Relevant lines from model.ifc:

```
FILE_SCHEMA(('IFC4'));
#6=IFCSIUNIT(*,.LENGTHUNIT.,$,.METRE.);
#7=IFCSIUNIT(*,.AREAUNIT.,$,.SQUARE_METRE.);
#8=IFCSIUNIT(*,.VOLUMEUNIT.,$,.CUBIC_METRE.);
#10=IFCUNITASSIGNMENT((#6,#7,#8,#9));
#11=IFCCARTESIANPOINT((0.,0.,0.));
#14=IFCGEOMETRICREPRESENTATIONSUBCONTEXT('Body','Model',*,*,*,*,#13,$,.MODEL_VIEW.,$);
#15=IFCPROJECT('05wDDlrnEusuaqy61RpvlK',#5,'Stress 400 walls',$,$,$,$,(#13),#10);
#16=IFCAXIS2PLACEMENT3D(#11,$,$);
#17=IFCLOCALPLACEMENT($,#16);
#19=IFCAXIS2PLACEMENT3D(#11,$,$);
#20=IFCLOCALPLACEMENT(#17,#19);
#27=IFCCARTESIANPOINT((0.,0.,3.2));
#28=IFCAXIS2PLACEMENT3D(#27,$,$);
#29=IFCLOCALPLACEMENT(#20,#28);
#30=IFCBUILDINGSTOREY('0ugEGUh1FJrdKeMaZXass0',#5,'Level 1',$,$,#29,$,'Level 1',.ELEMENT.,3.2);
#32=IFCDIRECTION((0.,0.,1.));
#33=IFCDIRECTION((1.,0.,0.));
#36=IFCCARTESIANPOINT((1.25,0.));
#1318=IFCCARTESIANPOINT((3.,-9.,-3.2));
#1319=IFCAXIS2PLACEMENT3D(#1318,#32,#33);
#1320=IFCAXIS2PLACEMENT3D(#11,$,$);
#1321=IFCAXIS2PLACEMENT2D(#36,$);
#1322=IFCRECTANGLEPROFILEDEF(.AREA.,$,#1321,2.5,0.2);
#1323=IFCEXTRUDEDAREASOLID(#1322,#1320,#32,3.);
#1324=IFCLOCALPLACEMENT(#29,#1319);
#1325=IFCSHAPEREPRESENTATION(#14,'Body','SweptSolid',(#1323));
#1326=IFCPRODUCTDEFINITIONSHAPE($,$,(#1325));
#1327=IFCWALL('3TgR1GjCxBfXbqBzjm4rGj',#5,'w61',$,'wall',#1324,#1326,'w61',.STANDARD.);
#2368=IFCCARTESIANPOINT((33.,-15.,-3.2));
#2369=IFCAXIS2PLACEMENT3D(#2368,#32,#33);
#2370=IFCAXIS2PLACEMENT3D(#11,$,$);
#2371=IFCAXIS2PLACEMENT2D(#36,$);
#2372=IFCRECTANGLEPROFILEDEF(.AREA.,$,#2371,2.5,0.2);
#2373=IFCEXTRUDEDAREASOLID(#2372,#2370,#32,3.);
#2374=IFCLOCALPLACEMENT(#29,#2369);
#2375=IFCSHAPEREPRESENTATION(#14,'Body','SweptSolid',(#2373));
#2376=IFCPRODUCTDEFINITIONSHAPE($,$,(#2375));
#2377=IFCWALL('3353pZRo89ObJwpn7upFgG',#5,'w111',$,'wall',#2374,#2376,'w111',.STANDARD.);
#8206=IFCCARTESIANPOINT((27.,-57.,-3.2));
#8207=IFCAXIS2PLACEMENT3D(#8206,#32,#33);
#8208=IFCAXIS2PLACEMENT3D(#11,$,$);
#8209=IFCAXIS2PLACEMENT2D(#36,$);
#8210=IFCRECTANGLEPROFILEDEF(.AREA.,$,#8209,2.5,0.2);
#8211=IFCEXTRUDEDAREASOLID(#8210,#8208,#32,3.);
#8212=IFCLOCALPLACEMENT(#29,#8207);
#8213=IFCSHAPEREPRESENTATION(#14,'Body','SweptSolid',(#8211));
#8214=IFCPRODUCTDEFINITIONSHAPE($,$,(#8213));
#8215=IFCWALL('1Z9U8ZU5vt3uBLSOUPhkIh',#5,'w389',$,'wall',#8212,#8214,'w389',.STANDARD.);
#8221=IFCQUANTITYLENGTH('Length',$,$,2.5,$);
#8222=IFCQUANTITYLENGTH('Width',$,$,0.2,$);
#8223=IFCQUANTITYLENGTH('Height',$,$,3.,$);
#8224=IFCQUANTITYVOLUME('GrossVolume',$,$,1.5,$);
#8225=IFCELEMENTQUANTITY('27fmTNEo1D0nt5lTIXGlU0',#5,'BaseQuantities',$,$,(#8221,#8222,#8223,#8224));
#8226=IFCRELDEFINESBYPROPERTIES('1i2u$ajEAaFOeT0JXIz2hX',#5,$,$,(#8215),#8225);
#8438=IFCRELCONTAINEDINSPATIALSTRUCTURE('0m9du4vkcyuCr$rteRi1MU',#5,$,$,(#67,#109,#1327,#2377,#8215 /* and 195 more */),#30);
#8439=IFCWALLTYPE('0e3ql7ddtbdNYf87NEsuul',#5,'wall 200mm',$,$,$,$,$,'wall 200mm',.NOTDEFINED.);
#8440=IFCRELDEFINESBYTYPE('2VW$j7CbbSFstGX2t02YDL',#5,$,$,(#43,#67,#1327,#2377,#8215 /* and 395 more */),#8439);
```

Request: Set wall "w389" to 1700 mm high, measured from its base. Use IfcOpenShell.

```python
import ifcopenshell
import ifcopenshell.api.pset
import ifcopenshell.geom
import ifcopenshell.util.element
import ifcopenshell.util.representation
import ifcopenshell.util.shape
import ifcopenshell.util.unit

model = ifcopenshell.open("model.ifc")
unit_scale = ifcopenshell.util.unit.calculate_unit_scale(model)
volume_scale = ifcopenshell.util.unit.calculate_unit_scale(model, "VOLUMEUNIT")
settings = ifcopenshell.geom.settings()


def volume(element):
    """Net volume in cubic metres, openings subtracted."""
    shape = ifcopenshell.geom.create_shape(settings, element)
    return ifcopenshell.util.shape.get_volume(shape.geometry)


wall = model.by_guid("1Z9U8ZU5vt3uBLSOUPhkIh")
before = volume(wall)

body = ifcopenshell.util.representation.get_representation(wall, "Model", "Body")
solid = body.Items[0]
old_height = solid.Depth
solid.Depth = 1.7 / unit_scale
after = volume(wall)

# Update the stored height, areas and volumes.
qto = model.by_id(ifcopenshell.util.element.get_pset(wall, "BaseQuantities", should_inherit=False)["id"])
ifcopenshell.api.pset.edit_qto(model, qto=qto, properties={
    "Height": solid.Depth,
    "GrossVolume": ifcopenshell.util.element.get_pset(wall, "BaseQuantities", "GrossVolume") * solid.Depth / old_height,
})

print(f"height {old_height:g} -> {solid.Depth:g}, volume {before:.3f} -> {after:.3f} m3")

model.write("model-out.ifc")
```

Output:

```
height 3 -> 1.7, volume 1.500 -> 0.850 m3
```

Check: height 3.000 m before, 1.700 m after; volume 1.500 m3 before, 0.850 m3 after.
